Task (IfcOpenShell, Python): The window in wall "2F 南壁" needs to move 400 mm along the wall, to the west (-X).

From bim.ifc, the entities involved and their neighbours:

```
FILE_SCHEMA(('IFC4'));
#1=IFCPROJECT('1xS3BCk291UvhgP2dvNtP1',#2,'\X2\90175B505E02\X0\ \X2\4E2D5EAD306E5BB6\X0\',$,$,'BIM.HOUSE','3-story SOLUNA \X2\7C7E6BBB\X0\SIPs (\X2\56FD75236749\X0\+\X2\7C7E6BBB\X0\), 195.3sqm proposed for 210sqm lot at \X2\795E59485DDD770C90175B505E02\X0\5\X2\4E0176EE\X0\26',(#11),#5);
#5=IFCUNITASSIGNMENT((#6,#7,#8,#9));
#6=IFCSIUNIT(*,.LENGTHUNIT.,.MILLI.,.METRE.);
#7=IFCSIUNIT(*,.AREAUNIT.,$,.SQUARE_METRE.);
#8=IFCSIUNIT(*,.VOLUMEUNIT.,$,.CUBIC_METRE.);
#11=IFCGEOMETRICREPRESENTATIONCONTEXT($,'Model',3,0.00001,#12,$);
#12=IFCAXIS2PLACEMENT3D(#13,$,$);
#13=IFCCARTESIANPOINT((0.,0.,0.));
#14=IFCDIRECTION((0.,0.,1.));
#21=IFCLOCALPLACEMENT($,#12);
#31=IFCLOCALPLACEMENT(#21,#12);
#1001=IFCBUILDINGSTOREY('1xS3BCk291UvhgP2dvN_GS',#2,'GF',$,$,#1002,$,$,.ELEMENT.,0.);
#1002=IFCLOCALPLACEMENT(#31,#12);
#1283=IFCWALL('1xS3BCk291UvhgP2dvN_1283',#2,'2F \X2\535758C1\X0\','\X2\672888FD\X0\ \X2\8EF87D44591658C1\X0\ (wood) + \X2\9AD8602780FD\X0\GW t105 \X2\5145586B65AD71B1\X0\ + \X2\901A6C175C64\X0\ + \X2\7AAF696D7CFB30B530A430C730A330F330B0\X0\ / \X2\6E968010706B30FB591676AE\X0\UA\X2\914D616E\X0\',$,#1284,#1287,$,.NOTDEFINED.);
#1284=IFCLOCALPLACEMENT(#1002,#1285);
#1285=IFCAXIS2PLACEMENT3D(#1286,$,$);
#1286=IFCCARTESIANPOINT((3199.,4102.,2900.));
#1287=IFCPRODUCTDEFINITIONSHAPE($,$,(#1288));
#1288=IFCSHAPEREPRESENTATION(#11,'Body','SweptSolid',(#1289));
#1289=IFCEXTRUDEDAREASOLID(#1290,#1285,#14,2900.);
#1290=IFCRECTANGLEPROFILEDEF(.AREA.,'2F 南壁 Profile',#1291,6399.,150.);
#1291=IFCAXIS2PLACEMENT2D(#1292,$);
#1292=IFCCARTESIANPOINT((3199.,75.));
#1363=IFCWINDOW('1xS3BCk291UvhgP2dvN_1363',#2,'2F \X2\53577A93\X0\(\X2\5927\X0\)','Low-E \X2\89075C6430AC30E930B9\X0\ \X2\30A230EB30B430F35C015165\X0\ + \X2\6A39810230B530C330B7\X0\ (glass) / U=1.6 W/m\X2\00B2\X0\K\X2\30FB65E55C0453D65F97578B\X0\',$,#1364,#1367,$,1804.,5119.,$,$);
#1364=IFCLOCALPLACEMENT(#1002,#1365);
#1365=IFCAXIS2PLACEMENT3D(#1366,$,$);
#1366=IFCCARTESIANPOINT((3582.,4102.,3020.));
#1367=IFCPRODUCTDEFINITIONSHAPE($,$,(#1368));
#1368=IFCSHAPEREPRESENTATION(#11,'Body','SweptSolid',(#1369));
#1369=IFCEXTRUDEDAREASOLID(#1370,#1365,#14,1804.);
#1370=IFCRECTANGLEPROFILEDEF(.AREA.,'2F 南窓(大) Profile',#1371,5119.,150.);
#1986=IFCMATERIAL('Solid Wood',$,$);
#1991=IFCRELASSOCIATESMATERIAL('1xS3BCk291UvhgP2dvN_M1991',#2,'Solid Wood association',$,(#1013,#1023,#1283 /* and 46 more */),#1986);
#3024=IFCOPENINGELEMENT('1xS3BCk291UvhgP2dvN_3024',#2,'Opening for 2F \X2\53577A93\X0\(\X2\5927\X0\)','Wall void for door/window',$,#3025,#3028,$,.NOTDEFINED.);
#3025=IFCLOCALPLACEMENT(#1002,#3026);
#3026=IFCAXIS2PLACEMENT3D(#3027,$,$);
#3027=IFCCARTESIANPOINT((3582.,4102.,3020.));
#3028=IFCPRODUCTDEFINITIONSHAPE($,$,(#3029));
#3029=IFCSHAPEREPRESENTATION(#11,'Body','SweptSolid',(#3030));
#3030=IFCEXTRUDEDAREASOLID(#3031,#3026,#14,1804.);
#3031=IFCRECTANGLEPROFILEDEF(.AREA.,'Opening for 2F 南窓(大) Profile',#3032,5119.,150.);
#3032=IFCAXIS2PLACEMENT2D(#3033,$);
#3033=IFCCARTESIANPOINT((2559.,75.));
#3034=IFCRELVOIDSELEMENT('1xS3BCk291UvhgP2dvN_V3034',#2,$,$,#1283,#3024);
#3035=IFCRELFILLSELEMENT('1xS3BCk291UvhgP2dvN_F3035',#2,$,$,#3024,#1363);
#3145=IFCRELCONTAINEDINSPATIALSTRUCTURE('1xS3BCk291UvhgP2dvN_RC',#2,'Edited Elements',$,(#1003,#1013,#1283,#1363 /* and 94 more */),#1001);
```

```python
import ifcopenshell
import ifcopenshell.api.geometry
import ifcopenshell.util.placement
import ifcopenshell.util.unit

model = ifcopenshell.open("bim.ifc")
unit_scale = ifcopenshell.util.unit.calculate_unit_scale(model)

window = model.by_guid("1xS3BCk291UvhgP2dvN_1363")
opening = window.FillsVoids[0].RelatingOpeningElement
wall = opening.VoidsElements[0].RelatingBuildingElement

wall_matrix = ifcopenshell.util.placement.get_local_placement(wall.ObjectPlacement)
shift = wall_matrix[:3, 0] * -0.4 / unit_scale
before = ifcopenshell.util.placement.get_local_placement(window.ObjectPlacement)[:3, 3].copy()

# The window is not placed relative to its opening, so move both.
for product in (opening, window):
    matrix = ifcopenshell.util.placement.get_local_placement(product.ObjectPlacement)
    matrix[:3, 3] += shift
    ifcopenshell.api.geometry.edit_object_placement(model, product=product, matrix=matrix, is_si=False)

after = ifcopenshell.util.placement.get_local_placement(window.ObjectPlacement)[:3, 3]
print("window moved by", (after - before).round(3) + 0.0)

model.write("bim-out.ifc")
```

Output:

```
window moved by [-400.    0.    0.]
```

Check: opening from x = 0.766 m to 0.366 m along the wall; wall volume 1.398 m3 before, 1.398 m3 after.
